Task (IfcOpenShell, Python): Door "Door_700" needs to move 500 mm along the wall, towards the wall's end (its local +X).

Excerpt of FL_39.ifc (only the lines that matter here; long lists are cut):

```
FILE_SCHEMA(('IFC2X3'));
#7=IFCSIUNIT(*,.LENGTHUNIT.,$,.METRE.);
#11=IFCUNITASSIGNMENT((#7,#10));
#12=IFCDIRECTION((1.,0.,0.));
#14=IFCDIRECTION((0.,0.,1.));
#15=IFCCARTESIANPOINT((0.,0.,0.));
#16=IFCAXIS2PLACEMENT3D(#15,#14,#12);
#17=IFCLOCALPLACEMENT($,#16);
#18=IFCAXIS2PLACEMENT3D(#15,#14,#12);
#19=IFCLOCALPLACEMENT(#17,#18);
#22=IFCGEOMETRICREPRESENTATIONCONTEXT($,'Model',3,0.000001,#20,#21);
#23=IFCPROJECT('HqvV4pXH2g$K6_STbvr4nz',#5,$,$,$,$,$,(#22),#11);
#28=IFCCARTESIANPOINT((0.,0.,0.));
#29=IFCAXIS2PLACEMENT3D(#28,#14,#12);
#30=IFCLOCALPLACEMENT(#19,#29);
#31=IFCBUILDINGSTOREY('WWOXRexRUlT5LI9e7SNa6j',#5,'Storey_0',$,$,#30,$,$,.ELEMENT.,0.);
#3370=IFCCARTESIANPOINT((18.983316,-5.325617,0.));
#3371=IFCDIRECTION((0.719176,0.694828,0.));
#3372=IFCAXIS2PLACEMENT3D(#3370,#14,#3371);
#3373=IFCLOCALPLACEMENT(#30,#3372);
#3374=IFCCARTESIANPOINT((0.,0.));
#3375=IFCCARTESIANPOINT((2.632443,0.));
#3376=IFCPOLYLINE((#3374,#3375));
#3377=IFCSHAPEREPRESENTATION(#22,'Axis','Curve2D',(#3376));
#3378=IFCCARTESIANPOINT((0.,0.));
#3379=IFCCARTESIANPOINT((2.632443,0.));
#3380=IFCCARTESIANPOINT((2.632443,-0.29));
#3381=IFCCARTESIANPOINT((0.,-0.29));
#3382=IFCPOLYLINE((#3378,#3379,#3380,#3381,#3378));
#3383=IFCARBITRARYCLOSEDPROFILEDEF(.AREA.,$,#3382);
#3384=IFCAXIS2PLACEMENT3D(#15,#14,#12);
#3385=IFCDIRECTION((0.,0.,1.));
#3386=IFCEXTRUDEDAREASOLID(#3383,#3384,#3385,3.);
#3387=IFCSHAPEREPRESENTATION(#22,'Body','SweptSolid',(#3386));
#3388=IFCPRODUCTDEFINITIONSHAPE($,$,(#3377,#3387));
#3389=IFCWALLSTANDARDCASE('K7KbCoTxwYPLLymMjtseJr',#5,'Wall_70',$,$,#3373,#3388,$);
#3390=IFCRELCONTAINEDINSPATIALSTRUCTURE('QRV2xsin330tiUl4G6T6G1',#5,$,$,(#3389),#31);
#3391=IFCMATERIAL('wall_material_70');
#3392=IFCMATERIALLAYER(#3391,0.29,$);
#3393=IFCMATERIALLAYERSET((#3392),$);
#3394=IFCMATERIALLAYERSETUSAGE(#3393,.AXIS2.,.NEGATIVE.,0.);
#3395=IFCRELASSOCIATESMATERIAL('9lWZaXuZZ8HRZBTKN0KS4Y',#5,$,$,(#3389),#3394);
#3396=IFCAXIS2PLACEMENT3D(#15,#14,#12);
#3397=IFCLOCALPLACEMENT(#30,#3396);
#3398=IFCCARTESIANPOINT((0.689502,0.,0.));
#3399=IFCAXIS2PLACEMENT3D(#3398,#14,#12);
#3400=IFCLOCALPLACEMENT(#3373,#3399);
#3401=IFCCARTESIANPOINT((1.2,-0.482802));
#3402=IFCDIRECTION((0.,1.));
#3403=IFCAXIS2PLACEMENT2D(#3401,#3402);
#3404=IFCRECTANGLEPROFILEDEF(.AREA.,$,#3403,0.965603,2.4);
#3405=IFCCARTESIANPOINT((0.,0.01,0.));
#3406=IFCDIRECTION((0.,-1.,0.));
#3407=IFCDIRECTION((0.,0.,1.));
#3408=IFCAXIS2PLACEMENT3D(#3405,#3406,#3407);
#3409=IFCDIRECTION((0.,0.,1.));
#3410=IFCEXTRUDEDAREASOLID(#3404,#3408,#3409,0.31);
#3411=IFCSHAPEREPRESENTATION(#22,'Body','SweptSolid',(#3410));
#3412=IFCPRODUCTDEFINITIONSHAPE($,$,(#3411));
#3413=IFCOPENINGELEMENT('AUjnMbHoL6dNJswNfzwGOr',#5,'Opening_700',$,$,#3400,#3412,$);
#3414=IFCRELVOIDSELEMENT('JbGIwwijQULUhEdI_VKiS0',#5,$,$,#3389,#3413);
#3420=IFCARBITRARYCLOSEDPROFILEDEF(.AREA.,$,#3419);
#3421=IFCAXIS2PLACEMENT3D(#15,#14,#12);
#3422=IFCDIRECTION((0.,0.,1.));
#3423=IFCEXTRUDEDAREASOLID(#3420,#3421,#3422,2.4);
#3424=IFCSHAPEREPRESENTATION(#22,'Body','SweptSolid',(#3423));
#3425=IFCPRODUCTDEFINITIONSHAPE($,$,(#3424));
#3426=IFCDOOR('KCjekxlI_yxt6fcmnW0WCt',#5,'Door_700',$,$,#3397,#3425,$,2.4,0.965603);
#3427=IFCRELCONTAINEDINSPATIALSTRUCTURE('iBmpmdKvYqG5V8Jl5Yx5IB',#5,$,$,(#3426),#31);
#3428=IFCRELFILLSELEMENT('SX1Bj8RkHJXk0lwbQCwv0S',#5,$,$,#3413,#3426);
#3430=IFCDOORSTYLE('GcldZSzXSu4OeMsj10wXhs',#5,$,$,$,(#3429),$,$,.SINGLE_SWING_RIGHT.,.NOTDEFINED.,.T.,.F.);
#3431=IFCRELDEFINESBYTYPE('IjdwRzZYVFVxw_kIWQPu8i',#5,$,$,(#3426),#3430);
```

```python
import ifcopenshell
import ifcopenshell.api.geometry
import ifcopenshell.util.placement
import ifcopenshell.util.unit

model = ifcopenshell.open("FL_39.ifc")
unit_scale = ifcopenshell.util.unit.calculate_unit_scale(model)

door = model.by_id(3426)
opening = door.FillsVoids[0].RelatingOpeningElement
wall = opening.VoidsElements[0].RelatingBuildingElement

wall_matrix = ifcopenshell.util.placement.get_local_placement(wall.ObjectPlacement)
shift = wall_matrix[:3, 0] * 0.5 / unit_scale
before = ifcopenshell.util.placement.get_local_placement(door.ObjectPlacement)[:3, 3].copy()

# The door is not placed relative to its opening, so move both.
for product in (opening, door):
    matrix = ifcopenshell.util.placement.get_local_placement(product.ObjectPlacement)
    matrix[:3, 3] += shift
    ifcopenshell.api.geometry.edit_object_placement(model, product=product, matrix=matrix, is_si=False)

after = ifcopenshell.util.placement.get_local_placement(door.ObjectPlacement)[:3, 3]
print("door moved by", (after - before).round(3) + 0.0)

model.write("FL_39_rev.ifc")
```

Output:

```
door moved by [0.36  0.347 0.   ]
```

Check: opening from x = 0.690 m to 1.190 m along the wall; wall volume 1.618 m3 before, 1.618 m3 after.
